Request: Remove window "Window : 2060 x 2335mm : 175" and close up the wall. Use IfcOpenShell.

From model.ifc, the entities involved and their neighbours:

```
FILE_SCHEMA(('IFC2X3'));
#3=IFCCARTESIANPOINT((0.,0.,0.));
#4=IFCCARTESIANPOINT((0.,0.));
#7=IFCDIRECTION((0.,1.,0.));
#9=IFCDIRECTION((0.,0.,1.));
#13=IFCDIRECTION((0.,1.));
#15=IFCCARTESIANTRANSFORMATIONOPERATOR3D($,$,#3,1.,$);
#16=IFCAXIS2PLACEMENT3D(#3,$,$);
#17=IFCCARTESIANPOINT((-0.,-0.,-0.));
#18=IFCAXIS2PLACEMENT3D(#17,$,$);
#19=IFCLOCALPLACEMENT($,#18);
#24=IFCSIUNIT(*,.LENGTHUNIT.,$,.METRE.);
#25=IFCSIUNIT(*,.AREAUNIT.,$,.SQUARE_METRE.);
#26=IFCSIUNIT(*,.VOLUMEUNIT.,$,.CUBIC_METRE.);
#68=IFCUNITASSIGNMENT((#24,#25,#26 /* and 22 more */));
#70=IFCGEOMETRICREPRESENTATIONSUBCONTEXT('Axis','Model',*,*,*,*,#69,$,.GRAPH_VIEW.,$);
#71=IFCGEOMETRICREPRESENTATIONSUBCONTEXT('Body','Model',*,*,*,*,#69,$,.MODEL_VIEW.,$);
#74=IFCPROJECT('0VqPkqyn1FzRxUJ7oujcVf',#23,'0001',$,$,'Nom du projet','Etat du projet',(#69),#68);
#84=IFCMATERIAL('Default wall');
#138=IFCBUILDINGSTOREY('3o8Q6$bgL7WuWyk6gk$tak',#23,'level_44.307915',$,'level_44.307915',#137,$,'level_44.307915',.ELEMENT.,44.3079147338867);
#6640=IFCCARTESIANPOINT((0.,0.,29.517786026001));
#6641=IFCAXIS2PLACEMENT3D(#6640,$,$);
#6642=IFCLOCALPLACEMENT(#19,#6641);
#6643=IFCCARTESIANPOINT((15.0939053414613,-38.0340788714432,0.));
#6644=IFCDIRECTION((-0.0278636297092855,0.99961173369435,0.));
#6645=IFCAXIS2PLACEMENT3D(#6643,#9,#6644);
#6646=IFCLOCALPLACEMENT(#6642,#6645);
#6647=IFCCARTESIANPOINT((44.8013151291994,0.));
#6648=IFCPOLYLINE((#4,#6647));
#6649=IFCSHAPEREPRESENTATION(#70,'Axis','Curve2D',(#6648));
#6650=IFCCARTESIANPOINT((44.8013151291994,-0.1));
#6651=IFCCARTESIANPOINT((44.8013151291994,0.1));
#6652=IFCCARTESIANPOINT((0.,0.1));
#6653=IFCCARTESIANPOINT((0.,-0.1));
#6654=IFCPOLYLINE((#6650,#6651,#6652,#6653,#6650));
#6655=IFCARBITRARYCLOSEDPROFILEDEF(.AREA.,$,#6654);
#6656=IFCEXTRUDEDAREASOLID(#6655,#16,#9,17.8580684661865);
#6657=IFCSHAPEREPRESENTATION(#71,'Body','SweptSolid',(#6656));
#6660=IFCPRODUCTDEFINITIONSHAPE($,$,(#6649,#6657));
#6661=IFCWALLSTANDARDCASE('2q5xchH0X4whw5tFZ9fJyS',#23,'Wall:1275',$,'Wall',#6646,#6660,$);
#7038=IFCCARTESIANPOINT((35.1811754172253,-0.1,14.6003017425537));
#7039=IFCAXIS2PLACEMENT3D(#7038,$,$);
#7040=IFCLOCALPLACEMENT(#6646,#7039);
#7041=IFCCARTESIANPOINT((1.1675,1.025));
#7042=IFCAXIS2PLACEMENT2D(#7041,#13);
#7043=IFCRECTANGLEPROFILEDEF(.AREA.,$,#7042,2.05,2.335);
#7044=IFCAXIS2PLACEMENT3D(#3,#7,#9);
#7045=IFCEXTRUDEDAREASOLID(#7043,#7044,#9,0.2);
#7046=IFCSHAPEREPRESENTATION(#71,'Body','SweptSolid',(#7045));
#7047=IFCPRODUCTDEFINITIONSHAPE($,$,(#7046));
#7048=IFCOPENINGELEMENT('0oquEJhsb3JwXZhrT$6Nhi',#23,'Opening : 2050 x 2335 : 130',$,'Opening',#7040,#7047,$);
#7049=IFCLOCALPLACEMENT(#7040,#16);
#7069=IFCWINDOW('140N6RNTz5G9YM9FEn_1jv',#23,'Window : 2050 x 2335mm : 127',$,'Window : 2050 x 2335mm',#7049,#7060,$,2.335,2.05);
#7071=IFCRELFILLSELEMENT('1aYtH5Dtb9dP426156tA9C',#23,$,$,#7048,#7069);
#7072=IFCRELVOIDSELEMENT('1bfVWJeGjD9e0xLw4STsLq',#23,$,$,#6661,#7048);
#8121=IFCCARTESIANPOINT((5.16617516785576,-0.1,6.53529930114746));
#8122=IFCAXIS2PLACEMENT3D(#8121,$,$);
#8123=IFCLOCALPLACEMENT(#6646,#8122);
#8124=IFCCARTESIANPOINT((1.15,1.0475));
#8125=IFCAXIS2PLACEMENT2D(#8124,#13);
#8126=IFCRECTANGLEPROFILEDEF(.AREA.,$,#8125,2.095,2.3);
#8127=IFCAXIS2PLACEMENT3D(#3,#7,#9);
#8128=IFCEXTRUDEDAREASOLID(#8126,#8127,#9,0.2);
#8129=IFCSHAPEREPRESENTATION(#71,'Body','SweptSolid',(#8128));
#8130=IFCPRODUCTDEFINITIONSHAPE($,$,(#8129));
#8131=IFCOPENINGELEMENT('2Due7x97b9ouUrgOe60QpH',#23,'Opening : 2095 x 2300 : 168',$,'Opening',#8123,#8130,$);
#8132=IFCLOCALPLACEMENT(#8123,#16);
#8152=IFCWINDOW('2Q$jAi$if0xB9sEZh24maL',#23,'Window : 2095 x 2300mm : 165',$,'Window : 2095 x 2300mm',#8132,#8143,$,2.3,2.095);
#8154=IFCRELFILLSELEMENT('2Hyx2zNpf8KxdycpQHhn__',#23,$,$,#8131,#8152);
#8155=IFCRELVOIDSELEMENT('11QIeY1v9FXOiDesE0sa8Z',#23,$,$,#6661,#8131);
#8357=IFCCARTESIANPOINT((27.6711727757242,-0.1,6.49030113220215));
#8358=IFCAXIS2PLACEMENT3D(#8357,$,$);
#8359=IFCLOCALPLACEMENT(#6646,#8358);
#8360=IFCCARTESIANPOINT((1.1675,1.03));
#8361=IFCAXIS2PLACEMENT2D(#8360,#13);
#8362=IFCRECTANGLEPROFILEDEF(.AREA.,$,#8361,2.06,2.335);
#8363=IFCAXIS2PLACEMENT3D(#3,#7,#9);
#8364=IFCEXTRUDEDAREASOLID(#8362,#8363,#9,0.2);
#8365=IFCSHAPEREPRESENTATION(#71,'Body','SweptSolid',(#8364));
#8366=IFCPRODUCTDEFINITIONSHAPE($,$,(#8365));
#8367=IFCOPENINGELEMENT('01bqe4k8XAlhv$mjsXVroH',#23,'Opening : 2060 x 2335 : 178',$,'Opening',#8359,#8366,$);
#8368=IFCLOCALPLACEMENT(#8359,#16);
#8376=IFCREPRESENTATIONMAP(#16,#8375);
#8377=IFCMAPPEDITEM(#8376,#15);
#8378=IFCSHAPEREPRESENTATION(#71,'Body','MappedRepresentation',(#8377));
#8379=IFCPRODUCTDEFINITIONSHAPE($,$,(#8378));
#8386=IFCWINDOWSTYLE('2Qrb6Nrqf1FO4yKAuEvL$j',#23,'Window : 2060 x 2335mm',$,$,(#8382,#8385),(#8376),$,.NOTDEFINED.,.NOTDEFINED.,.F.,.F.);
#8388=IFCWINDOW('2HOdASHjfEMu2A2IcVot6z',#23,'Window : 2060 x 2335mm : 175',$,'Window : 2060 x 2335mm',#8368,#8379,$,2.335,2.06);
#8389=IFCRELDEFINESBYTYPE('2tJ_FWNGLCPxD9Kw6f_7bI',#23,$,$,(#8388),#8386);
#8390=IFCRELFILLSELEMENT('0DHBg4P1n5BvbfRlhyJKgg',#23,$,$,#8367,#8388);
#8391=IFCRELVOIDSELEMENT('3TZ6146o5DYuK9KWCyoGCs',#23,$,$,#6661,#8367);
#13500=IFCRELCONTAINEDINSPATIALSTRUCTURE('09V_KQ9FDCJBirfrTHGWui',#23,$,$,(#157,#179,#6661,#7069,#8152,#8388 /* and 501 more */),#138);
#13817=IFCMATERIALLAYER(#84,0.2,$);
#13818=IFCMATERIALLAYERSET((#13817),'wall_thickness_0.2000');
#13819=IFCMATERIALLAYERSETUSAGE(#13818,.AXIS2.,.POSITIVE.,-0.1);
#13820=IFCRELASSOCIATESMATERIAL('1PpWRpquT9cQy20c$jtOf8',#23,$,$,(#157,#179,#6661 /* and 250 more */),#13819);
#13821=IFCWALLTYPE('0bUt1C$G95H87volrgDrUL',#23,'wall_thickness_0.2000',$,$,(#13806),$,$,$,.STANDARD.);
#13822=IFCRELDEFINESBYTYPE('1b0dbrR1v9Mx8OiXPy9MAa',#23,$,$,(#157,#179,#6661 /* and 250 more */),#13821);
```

```python
import ifcopenshell
import ifcopenshell.api.feature
import ifcopenshell.api.root
import ifcopenshell.geom
import ifcopenshell.util.shape

model = ifcopenshell.open("model.ifc")
settings = ifcopenshell.geom.settings()


def volume(element):
    """Net volume in cubic metres, openings subtracted."""
    shape = ifcopenshell.geom.create_shape(settings, element)
    return ifcopenshell.util.shape.get_volume(shape.geometry)


window = model.by_id(8388)
opening = window.FillsVoids[0].RelatingOpeningElement
wall = opening.VoidsElements[0].RelatingBuildingElement
before = volume(wall)

ifcopenshell.api.root.remove_product(model, product=window)
ifcopenshell.api.feature.remove_feature(model, feature=opening)

after = volume(wall)

print(f"wall volume {before:.3f} -> {after:.3f} m3")

model.write("model_updated.ifc")
```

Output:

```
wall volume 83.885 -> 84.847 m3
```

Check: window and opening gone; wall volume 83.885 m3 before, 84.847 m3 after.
